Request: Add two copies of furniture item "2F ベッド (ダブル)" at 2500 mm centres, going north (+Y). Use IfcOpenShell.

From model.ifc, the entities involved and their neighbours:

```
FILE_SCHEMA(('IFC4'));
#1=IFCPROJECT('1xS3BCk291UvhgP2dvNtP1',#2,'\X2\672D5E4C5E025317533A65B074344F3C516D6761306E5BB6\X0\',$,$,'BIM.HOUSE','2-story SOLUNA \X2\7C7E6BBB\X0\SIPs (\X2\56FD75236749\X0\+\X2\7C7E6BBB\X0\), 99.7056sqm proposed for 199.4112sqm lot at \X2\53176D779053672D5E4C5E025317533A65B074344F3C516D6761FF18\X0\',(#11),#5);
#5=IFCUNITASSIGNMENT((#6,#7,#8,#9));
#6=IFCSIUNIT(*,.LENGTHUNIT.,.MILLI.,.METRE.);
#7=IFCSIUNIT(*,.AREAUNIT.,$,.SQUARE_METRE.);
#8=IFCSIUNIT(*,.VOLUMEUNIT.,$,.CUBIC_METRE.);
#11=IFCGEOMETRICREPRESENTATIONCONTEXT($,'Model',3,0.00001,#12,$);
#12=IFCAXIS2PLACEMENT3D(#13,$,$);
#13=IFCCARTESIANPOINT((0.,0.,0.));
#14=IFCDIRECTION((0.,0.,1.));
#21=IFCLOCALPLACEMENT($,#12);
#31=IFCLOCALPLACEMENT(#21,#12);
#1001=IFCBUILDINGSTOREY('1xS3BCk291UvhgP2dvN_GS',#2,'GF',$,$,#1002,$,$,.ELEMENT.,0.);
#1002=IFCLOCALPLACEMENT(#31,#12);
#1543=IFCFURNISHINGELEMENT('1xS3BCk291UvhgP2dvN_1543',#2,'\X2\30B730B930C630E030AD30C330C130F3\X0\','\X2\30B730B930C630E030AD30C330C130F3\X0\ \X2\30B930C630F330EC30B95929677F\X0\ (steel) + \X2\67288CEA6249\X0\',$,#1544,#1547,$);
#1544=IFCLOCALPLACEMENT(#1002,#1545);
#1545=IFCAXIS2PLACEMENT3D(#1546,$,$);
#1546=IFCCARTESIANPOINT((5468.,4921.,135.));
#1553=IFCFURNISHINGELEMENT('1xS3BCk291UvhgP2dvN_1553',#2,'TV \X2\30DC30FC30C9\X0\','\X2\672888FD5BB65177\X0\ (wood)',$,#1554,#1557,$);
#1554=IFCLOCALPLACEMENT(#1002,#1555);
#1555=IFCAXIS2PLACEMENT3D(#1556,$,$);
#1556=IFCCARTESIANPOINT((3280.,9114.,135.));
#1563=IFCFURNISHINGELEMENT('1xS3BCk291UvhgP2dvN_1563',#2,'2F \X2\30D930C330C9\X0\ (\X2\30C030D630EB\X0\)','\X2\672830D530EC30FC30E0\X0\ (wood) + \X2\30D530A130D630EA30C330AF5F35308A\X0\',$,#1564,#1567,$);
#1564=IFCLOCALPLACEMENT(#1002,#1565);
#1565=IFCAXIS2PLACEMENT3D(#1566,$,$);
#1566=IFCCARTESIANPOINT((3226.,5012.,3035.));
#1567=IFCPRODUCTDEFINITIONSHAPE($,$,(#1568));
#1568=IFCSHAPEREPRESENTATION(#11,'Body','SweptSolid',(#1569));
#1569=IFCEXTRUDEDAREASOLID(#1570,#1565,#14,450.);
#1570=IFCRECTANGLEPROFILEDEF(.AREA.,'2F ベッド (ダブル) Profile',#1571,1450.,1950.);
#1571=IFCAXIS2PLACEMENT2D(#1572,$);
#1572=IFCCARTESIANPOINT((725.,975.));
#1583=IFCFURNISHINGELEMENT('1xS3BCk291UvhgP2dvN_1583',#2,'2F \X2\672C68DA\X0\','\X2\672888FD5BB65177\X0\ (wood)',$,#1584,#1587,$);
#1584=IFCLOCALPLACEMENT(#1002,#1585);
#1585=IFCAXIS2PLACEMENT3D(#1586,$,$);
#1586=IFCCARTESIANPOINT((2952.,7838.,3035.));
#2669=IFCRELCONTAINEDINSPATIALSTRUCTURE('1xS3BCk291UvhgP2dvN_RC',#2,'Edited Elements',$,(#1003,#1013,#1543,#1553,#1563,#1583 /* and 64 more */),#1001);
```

```python
import numpy as np
import ifcopenshell
import ifcopenshell.api.geometry
import ifcopenshell.api.root
import ifcopenshell.util.element
import ifcopenshell.util.placement

model = ifcopenshell.open("model.ifc")


def reuse_history(source, copy):
    """copy_class also copies each property set's owner history, people and application; keep the originals."""
    for rel in copy.IsDefinedBy:
        if rel.is_a("IfcRelDefinesByProperties") and (history := rel.RelatingPropertyDefinition.OwnerHistory):
            rel.RelatingPropertyDefinition.OwnerHistory = source.OwnerHistory
            ifcopenshell.util.element.remove_deep2(model, history)


source = model.by_id(1563)
base = ifcopenshell.util.placement.get_local_placement(source.ObjectPlacement)
step = np.array([0.0, 1.0, 0.0]) * 2500.0

for i in range(1, 3):
    copy = ifcopenshell.api.root.copy_class(model, product=source)
    copy.Representation = ifcopenshell.util.element.copy_deep(
        model, source.Representation, exclude=["IfcGeometricRepresentationContext", "IfcRepresentationMap"]
    )
    reuse_history(source, copy)
    matrix = base.copy()
    matrix[:3, 3] += i * step
    print("added at", matrix[:3, 3].round(3) + 0.0)
    ifcopenshell.api.geometry.edit_object_placement(model, product=copy, matrix=matrix, is_si=False)

model.write("model_updated.ifc")
```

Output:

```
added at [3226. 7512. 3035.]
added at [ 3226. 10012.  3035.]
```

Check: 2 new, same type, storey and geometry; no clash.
